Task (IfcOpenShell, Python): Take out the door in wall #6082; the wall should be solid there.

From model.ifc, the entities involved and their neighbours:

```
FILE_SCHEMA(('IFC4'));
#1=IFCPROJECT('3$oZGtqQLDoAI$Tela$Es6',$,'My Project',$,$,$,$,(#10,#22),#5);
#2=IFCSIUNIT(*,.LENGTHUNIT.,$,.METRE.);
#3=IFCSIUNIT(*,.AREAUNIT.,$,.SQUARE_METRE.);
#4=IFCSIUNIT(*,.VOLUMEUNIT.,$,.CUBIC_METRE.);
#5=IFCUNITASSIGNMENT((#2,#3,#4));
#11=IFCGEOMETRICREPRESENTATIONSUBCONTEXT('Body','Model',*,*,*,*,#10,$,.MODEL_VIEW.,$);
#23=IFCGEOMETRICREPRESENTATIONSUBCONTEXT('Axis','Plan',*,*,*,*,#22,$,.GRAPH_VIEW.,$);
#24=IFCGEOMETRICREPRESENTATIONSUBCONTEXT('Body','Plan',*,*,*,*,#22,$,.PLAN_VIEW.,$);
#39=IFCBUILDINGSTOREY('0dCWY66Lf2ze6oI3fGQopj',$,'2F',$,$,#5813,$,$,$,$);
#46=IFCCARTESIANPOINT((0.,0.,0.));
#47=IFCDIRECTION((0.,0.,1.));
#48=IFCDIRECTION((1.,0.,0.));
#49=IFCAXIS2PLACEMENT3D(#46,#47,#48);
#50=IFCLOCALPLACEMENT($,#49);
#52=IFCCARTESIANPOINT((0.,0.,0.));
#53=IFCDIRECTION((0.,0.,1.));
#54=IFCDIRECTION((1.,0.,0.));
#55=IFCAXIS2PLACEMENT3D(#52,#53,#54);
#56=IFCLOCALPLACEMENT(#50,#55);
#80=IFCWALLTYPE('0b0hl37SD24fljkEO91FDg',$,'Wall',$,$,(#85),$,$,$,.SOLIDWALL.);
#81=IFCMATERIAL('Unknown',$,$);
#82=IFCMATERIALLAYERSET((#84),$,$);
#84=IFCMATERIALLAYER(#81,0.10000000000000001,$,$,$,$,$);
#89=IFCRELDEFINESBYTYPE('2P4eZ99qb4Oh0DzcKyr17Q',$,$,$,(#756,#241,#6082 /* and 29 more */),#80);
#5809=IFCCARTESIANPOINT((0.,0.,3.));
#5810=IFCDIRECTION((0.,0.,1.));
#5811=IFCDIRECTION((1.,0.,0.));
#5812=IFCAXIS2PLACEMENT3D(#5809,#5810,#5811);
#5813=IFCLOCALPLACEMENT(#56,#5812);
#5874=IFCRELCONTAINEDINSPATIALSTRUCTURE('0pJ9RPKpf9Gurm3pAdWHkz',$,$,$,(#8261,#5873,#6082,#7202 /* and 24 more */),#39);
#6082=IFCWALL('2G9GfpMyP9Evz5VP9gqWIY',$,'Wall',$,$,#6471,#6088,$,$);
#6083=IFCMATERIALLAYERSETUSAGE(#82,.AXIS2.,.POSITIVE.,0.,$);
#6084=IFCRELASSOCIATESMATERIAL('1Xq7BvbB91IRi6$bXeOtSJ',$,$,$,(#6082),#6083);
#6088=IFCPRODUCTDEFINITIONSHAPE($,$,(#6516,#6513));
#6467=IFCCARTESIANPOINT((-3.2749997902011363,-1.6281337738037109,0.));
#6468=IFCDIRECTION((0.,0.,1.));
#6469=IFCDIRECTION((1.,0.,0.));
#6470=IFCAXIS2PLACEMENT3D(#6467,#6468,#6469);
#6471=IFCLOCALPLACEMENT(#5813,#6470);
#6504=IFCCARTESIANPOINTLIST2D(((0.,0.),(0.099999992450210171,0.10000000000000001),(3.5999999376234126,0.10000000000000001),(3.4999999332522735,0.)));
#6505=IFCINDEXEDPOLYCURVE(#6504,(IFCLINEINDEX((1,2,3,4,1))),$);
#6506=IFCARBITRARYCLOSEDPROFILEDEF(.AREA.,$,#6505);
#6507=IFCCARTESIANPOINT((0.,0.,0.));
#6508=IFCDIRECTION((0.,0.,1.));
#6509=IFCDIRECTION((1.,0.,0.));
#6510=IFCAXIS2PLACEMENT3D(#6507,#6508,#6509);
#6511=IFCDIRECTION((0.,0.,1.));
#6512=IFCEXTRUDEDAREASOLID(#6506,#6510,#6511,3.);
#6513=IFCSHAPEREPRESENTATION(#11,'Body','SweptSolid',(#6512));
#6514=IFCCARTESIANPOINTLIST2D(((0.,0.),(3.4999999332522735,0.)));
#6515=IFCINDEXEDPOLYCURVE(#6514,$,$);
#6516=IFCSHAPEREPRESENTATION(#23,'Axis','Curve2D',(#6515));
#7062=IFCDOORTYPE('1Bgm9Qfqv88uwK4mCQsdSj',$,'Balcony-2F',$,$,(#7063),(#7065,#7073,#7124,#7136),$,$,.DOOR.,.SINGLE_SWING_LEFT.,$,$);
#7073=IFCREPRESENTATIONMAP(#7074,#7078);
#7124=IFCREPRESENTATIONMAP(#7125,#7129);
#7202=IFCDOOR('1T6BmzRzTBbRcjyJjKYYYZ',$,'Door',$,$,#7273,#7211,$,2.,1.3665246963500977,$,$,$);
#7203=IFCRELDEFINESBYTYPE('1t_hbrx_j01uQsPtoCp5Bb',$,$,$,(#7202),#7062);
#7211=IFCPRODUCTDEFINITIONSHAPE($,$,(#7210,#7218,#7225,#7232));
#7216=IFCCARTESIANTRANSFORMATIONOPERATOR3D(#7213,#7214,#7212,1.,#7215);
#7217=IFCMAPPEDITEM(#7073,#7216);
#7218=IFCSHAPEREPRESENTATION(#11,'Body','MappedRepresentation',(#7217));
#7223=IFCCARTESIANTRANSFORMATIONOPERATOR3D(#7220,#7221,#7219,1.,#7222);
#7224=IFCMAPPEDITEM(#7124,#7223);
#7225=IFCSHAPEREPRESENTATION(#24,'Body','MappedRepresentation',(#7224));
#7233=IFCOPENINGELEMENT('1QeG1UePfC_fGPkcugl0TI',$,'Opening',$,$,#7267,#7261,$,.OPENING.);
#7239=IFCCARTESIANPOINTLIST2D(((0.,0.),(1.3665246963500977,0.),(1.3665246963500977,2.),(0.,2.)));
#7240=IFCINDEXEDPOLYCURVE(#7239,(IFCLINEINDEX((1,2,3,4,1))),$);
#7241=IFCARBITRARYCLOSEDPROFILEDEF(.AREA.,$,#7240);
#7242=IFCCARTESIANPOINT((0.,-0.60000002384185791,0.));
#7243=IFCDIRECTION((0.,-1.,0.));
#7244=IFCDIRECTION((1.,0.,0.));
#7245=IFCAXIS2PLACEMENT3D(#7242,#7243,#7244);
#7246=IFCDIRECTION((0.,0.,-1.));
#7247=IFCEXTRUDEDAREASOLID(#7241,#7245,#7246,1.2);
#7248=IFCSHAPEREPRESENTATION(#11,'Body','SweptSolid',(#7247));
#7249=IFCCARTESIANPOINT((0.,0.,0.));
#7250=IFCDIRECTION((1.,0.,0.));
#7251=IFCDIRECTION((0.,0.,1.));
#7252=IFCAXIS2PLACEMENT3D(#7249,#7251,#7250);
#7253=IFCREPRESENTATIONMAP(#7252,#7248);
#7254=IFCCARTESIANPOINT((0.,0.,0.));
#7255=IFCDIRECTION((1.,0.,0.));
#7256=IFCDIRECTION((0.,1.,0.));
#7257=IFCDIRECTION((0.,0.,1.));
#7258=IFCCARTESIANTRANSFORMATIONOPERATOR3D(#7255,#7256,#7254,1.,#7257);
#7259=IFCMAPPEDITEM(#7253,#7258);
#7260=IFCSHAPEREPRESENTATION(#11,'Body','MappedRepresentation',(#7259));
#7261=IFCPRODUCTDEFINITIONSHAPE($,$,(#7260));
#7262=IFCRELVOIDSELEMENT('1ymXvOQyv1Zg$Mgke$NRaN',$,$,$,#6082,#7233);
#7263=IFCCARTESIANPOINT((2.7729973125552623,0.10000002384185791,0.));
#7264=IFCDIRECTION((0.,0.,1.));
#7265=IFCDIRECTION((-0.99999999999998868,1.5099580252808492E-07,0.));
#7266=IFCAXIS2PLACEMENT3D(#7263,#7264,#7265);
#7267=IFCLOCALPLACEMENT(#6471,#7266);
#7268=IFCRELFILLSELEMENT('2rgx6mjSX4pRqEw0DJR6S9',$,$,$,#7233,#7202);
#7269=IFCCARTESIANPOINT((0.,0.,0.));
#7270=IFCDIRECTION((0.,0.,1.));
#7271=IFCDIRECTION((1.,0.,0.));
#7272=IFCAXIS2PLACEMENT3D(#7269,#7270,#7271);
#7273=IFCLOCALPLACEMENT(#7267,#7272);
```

```python
import ifcopenshell
import ifcopenshell.api.feature
import ifcopenshell.api.root
import ifcopenshell.geom
import ifcopenshell.util.shape

model = ifcopenshell.open("model.ifc")
settings = ifcopenshell.geom.settings()


def volume(element):
    """Net volume in cubic metres, openings subtracted."""
    shape = ifcopenshell.geom.create_shape(settings, element)
    return ifcopenshell.util.shape.get_volume(shape.geometry)


door = model.by_guid("1T6BmzRzTBbRcjyJjKYYYZ")
opening = door.FillsVoids[0].RelatingOpeningElement
wall = opening.VoidsElements[0].RelatingBuildingElement
before = volume(wall)

ifcopenshell.api.root.remove_product(model, product=door)
ifcopenshell.api.feature.remove_feature(model, feature=opening)

after = volume(wall)

print(f"wall volume {before:.3f} -> {after:.3f} m3")

model.write("model_edited.ifc")
```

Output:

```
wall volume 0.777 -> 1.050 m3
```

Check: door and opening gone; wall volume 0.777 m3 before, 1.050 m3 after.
